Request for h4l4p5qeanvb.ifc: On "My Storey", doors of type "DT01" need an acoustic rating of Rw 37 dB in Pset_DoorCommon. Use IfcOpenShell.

First a look at what the model holds.

```python
import ifcopenshell
import ifcopenshell.util.element

model = ifcopenshell.open("h4l4p5qeanvb.ifc")
print(model.schema)
storey = next(s for s in model.by_type("IfcBuildingStorey") if s.Name == "My Storey")
doors = [e for e in ifcopenshell.util.element.get_decomposition(storey) if e.is_a("IfcDoor")]
seen = {}
for e in doors:
    element_type = ifcopenshell.util.element.get_type(e)
    key = (element_type.Name if element_type != e and element_type else None, ifcopenshell.util.element.get_pset(e, "Pset_DoorCommon", "AcousticRating"))
    seen[key] = seen.get(key, 0) + 1
for (name, value), count in sorted(seen.items(), key=str):
    print(count, "x", name, "|", value)
```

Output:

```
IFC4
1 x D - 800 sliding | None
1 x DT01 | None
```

```python
import ifcopenshell
import ifcopenshell.api.pset
import ifcopenshell.util.element

model = ifcopenshell.open("h4l4p5qeanvb.ifc")

storey = next(s for s in model.by_type("IfcBuildingStorey") if s.Name == "My Storey")
doors = [e for e in ifcopenshell.util.element.get_decomposition(storey) if e.is_a("IfcDoor")]

count = 0
for e in doors:
    element_type = ifcopenshell.util.element.get_type(e)
    if element_type in (None, e) or element_type.Name != "DT01":
        continue
    # add_pset returns the element's existing set when there is one.
    pset = ifcopenshell.api.pset.add_pset(model, product=e, name="Pset_DoorCommon")
    ifcopenshell.api.pset.edit_pset(model, pset=pset, properties={"AcousticRating": "Rw 37 dB"})
    count += 1

print(count, "doors updated")

model.write("h4l4p5qeanvb_updated.ifc")
```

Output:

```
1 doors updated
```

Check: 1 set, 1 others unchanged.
